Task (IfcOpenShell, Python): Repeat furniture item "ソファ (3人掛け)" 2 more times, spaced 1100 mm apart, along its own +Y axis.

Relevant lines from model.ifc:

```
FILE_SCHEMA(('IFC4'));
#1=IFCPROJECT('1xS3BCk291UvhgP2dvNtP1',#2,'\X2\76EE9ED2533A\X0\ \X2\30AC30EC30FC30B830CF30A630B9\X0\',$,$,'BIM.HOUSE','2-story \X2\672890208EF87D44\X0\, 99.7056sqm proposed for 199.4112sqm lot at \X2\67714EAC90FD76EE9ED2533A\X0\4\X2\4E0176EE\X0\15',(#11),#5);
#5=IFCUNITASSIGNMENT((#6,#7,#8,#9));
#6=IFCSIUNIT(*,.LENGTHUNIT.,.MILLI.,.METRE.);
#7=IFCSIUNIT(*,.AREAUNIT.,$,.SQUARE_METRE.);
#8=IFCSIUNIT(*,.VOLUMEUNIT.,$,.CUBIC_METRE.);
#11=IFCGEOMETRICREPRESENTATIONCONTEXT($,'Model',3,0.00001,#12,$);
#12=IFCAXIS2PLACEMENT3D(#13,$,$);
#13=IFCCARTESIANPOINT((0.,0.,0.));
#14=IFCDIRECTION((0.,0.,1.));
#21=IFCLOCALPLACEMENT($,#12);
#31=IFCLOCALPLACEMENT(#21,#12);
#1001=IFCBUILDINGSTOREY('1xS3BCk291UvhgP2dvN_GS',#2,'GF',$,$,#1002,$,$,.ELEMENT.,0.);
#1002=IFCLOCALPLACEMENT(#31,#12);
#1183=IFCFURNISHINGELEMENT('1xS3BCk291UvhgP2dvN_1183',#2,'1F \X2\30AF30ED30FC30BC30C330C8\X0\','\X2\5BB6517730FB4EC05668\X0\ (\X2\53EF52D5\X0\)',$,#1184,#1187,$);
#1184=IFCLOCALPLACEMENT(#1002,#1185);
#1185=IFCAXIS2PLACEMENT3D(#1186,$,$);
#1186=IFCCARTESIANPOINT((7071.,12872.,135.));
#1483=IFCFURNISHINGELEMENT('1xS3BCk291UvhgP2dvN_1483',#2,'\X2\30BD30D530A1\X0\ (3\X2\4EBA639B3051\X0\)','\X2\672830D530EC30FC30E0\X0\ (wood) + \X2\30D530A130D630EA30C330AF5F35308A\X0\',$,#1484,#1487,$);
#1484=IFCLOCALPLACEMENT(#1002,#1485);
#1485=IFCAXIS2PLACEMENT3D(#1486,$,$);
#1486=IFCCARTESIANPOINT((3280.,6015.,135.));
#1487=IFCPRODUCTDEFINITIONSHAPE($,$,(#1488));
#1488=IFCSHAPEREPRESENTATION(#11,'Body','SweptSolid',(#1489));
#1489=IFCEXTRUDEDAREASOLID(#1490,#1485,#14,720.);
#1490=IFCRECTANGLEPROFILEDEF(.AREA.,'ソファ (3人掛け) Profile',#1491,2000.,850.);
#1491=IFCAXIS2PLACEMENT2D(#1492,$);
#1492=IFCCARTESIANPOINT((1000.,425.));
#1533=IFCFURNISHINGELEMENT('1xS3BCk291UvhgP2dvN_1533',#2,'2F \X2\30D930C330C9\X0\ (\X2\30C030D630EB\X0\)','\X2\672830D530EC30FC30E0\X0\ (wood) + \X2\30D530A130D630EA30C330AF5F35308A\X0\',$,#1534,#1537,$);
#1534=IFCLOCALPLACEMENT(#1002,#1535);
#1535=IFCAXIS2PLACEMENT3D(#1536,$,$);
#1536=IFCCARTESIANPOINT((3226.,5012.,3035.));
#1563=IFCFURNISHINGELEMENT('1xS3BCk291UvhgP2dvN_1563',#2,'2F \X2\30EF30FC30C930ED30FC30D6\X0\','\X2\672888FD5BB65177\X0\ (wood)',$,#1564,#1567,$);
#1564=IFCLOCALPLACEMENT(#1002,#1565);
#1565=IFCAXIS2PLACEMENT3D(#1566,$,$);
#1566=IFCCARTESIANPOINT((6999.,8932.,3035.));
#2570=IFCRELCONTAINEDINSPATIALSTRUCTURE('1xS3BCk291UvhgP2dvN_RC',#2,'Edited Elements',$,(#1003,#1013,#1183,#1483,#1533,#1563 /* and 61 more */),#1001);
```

```python
import ifcopenshell
import ifcopenshell.api.geometry
import ifcopenshell.api.root
import ifcopenshell.util.element
import ifcopenshell.util.placement
import ifcopenshell.util.unit

model = ifcopenshell.open("model.ifc")
unit_scale = ifcopenshell.util.unit.calculate_unit_scale(model)


def reuse_history(source, copy):
    """copy_class also copies each property set's owner history, people and application; keep the originals."""
    for rel in copy.IsDefinedBy:
        if rel.is_a("IfcRelDefinesByProperties") and (history := rel.RelatingPropertyDefinition.OwnerHistory):
            rel.RelatingPropertyDefinition.OwnerHistory = source.OwnerHistory
            ifcopenshell.util.element.remove_deep2(model, history)


source = model.by_guid("1xS3BCk291UvhgP2dvN_1483")
base = ifcopenshell.util.placement.get_local_placement(source.ObjectPlacement)
step = base[:3, 1] * 1.1 / unit_scale

for i in range(1, 3):
    copy = ifcopenshell.api.root.copy_class(model, product=source)
    copy.Representation = ifcopenshell.util.element.copy_deep(
        model, source.Representation, exclude=["IfcGeometricRepresentationContext", "IfcRepresentationMap"]
    )
    reuse_history(source, copy)
    matrix = base.copy()
    matrix[:3, 3] += i * step
    print("added at", matrix[:3, 3].round(3) + 0.0)
    ifcopenshell.api.geometry.edit_object_placement(model, product=copy, matrix=matrix, is_si=False)

model.write("model_updated.ifc")
```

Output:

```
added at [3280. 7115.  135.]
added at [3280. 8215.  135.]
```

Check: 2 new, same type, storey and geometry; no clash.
